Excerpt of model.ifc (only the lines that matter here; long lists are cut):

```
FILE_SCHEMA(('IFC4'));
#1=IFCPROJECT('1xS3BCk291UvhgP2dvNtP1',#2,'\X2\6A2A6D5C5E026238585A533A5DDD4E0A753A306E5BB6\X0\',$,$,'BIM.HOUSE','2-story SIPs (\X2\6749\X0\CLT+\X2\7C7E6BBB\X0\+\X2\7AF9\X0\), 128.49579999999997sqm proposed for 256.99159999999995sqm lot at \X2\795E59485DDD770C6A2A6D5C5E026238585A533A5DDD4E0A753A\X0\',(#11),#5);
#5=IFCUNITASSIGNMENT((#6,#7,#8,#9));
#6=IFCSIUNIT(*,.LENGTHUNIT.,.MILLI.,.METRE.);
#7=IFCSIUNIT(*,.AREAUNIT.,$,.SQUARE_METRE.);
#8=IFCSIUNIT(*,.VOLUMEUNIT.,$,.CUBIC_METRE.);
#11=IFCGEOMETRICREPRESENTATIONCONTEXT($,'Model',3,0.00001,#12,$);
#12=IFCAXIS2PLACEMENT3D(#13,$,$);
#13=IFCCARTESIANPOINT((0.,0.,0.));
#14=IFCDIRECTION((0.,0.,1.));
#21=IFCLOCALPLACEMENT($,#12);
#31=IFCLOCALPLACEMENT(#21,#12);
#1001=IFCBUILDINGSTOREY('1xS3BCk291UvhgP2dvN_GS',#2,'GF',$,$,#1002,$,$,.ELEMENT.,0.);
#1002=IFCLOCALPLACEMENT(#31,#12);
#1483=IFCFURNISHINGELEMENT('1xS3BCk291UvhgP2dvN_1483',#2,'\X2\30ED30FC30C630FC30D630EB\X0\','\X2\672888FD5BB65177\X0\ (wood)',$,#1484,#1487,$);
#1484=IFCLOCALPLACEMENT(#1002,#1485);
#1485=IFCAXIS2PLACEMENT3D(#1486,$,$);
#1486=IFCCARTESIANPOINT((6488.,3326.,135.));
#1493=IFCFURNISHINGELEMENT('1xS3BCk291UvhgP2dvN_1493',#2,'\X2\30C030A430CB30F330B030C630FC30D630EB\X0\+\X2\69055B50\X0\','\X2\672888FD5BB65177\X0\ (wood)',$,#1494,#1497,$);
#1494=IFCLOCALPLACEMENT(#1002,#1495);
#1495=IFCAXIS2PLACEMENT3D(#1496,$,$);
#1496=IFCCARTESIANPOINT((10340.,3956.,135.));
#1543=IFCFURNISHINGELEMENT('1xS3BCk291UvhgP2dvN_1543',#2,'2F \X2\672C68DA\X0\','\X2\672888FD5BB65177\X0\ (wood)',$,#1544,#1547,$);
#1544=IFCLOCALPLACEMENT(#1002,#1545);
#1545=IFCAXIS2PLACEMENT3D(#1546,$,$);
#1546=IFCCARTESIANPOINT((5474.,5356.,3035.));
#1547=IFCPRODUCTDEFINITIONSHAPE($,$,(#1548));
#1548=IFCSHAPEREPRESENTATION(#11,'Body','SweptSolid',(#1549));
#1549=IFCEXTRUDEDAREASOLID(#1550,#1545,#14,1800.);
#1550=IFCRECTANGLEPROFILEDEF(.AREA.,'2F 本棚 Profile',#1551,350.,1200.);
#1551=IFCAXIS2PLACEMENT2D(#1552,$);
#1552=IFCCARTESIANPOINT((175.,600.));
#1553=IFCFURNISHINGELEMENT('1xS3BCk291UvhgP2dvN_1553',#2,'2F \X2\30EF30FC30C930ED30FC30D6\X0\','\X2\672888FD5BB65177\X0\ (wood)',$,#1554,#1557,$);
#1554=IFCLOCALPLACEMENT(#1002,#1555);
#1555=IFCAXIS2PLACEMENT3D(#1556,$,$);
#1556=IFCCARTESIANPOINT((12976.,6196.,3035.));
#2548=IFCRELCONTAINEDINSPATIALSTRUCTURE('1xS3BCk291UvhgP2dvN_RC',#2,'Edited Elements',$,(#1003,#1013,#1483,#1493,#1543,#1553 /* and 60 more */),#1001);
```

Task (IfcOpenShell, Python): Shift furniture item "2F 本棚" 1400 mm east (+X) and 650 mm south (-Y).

```python
import ifcopenshell
import ifcopenshell.api.geometry
import ifcopenshell.util.placement
import ifcopenshell.util.unit

model = ifcopenshell.open("model.ifc")
unit_scale = ifcopenshell.util.unit.calculate_unit_scale(model)

item = model.by_guid("1xS3BCk291UvhgP2dvN_1543")
matrix = ifcopenshell.util.placement.get_local_placement(item.ObjectPlacement)
matrix[0, 3] += 1.4 / unit_scale
matrix[1, 3] -= 0.65 / unit_scale
ifcopenshell.api.geometry.edit_object_placement(model, product=item, matrix=matrix, is_si=False)

print(ifcopenshell.util.placement.get_local_placement(item.ObjectPlacement).round(3) + 0.0)

model.write("model_rev.ifc")
```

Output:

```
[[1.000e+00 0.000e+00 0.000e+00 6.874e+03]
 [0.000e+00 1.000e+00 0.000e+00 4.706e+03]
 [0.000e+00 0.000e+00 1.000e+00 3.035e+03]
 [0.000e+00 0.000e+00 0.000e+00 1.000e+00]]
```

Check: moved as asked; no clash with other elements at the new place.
